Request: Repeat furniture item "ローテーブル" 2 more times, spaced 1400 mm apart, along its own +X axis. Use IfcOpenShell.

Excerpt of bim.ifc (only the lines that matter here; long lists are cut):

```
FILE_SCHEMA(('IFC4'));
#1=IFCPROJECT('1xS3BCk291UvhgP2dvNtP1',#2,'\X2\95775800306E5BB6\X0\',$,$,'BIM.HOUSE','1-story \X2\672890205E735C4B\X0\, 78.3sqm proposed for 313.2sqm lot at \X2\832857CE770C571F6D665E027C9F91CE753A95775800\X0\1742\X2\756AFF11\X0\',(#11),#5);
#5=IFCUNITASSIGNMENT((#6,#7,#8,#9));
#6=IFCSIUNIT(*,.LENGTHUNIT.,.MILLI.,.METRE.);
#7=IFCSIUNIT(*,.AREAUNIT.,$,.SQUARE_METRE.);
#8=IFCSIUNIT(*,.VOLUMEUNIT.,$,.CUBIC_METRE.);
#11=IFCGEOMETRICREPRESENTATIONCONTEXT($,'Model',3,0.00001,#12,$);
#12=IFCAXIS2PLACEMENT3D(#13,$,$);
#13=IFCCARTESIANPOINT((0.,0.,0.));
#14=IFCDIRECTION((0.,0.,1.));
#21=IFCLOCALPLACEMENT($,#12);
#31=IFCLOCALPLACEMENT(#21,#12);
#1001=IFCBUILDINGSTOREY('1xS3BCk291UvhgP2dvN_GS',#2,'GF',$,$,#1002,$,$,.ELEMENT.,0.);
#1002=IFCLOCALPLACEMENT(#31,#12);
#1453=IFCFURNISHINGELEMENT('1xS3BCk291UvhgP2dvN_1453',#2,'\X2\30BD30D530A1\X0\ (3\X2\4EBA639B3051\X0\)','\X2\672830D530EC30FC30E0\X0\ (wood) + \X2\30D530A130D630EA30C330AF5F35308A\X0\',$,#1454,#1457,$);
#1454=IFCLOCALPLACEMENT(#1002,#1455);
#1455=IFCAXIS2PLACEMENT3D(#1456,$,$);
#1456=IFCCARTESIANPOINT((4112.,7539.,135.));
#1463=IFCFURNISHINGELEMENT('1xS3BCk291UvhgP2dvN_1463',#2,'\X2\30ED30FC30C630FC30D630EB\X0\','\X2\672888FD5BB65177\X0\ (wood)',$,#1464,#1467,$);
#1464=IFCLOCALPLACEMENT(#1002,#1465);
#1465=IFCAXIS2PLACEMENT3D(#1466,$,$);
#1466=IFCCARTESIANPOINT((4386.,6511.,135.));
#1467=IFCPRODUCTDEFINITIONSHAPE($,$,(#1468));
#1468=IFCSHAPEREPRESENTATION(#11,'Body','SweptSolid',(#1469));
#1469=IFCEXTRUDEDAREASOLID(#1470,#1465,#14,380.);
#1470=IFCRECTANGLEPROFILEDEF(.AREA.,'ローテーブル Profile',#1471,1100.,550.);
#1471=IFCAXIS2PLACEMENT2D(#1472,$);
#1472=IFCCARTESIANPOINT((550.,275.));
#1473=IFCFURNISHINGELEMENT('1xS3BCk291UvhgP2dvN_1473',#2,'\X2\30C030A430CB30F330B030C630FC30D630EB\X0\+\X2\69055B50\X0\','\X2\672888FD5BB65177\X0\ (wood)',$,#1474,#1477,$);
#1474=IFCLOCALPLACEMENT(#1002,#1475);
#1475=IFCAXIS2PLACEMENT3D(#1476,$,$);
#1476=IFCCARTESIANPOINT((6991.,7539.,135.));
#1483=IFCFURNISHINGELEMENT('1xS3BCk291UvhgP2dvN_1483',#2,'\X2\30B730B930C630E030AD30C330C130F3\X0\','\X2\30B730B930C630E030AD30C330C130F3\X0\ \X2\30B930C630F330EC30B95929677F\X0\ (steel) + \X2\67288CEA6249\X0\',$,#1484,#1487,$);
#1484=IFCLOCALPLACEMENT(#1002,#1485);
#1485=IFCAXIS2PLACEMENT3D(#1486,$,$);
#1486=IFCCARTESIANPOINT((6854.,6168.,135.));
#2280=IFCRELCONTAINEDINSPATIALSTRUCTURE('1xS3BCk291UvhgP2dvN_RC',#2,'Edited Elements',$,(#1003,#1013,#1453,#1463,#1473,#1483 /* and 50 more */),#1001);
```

```python
import ifcopenshell
import ifcopenshell.api.geometry
import ifcopenshell.api.root
import ifcopenshell.util.element
import ifcopenshell.util.placement

model = ifcopenshell.open("bim.ifc")


def reuse_history(source, copy):
    """copy_class also copies each property set's owner history, people and application; keep the originals."""
    for rel in copy.IsDefinedBy:
        if rel.is_a("IfcRelDefinesByProperties") and (history := rel.RelatingPropertyDefinition.OwnerHistory):
            rel.RelatingPropertyDefinition.OwnerHistory = source.OwnerHistory
            ifcopenshell.util.element.remove_deep2(model, history)


source = model.by_id(1463)
base = ifcopenshell.util.placement.get_local_placement(source.ObjectPlacement)
step = base[:3, 0] * 1400.0

for i in range(1, 3):
    copy = ifcopenshell.api.root.copy_class(model, product=source)
    copy.Representation = ifcopenshell.util.element.copy_deep(
        model, source.Representation, exclude=["IfcGeometricRepresentationContext", "IfcRepresentationMap"]
    )
    reuse_history(source, copy)
    matrix = base.copy()
    matrix[:3, 3] += i * step
    print("added at", matrix[:3, 3].round(3) + 0.0)
    ifcopenshell.api.geometry.edit_object_placement(model, product=copy, matrix=matrix, is_si=False)

model.write("bim-out.ifc")
```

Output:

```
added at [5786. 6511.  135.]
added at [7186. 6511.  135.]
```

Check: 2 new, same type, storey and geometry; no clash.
